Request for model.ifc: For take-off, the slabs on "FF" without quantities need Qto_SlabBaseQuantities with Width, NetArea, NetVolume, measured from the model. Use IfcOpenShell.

First a look at what the model holds.

```python
import ifcopenshell
import ifcopenshell.util.element
import ifcopenshell.util.unit

model = ifcopenshell.open("model.ifc")
print(model.schema)
for unit_type in ("LENGTHUNIT", "AREAUNIT", "VOLUMEUNIT"):
    print(unit_type, ifcopenshell.util.unit.calculate_unit_scale(model, unit_type))
storey = next(s for s in model.by_type("IfcBuildingStorey") if s.Name == "FF")
slabs = [e for e in ifcopenshell.util.element.get_decomposition(storey) if e.is_a("IfcSlab")]
for e in sorted(slabs, key=lambda e: e.id()):
    print(e.id(), e.is_a(), e.Name, list(ifcopenshell.util.element.get_psets(e, qtos_only=True)), sep=" | ")
```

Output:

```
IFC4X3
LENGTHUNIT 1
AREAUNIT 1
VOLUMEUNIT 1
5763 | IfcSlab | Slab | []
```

```python
import ifcopenshell
import ifcopenshell.api.pset
import ifcopenshell.geom
import ifcopenshell.util.element
import ifcopenshell.util.shape
import ifcopenshell.util.unit

model = ifcopenshell.open("model.ifc")
unit_scale = ifcopenshell.util.unit.calculate_unit_scale(model)
area_scale = ifcopenshell.util.unit.calculate_unit_scale(model, "AREAUNIT")
volume_scale = ifcopenshell.util.unit.calculate_unit_scale(model, "VOLUMEUNIT")
settings = ifcopenshell.geom.settings()

storey = next(s for s in model.by_type("IfcBuildingStorey") if s.Name == "FF")
slabs = [e for e in ifcopenshell.util.element.get_decomposition(storey) if e.is_a("IfcSlab")]

for e in sorted(slabs, key=lambda e: e.id()):
    if ifcopenshell.util.element.get_psets(e, qtos_only=True, should_inherit=False):
        continue
    # Geometry comes back in metres, in the element's own axes.
    shape = ifcopenshell.geom.create_shape(settings, e)
    values = {
        "Width": ifcopenshell.util.shape.get_z(shape.geometry) / unit_scale,
        "NetArea": ifcopenshell.util.shape.get_footprint_area(shape.geometry) / area_scale,
        "NetVolume": ifcopenshell.util.shape.get_volume(shape.geometry) / volume_scale,
    }
    qto = ifcopenshell.api.pset.add_qto(model, product=e, name="Qto_SlabBaseQuantities")
    ifcopenshell.api.pset.edit_qto(model, qto=qto, properties=values)
    print(e.id(), {k: round(v, 3) for k, v in values.items()})

model.write("model_updated.ifc")
```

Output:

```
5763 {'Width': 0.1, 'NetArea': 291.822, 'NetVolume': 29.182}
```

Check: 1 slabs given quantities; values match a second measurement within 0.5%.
